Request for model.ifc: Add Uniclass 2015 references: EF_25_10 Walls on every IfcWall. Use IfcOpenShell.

First a look at what the model holds.

```python
import ifcopenshell

model = ifcopenshell.open("model.ifc")
print(model.schema)
print("classifications:", [c.Name for c in model.by_type("IfcClassification")])
for ifc_class in ("IfcDoor", "IfcRoof", "IfcStair", "IfcWall", "IfcWindow"):
    print(ifc_class, len(model.by_type(ifc_class)))
```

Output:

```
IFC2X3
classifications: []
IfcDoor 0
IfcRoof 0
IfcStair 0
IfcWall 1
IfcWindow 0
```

```python
import ifcopenshell
import ifcopenshell.api.classification

model = ifcopenshell.open("model.ifc")

# IFC2X3 requires Source and Edition and has no link from the project to the system.
system = model.create_entity("IfcClassification", Source="NBS", Edition="2015", Name="Uniclass 2015")

codes = {
    "IfcWall": ("EF_25_10", "Walls"),
}
for ifc_class, (code, name) in codes.items():
    products = model.by_type(ifc_class)
    ifcopenshell.api.classification.add_reference(
        model, products=products, classification=system, identification=code, name=name
    )
    print(code, len(products))

model.write("model-out.ifc")
```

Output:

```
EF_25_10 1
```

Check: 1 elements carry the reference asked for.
